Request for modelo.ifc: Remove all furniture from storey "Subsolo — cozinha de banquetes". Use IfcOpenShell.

First a look at what the model holds.

```python
import ifcopenshell
import ifcopenshell.util.element

model = ifcopenshell.open("modelo.ifc")
print(model.schema)
storey = next(s for s in model.by_type("IfcBuildingStorey") if s.Name == "Subsolo — cozinha de banquetes")
furniture = [e for e in ifcopenshell.util.element.get_decomposition(storey) if e.is_a("IfcFurnishingElement")]
seen = {}
for e in furniture:
    element_type = ifcopenshell.util.element.get_type(e)
    name = element_type.Name if element_type not in (None, e) else None
    seen[name] = seen.get(name, 0) + 1
for name, count in sorted(seen.items(), key=str):
    print(count, "x", name)
```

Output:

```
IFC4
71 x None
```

```python
import ifcopenshell
import ifcopenshell.api.root
import ifcopenshell.util.element

model = ifcopenshell.open("modelo.ifc")

storey = next(s for s in model.by_type("IfcBuildingStorey") if s.Name == "Subsolo — cozinha de banquetes")
furniture = [e for e in ifcopenshell.util.element.get_decomposition(storey) if e.is_a("IfcFurnishingElement")]

for e in furniture:
    ifcopenshell.api.root.remove_product(model, product=e)
print(len(furniture), "removed")

model.write("modelo_v2.ifc")
```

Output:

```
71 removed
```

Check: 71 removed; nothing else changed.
